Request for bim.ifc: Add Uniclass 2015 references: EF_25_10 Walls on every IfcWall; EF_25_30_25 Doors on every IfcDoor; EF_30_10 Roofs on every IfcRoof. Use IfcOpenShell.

First a look at what the model holds.

```python
import ifcopenshell

model = ifcopenshell.open("bim.ifc")
print(model.schema)
print("classifications:", [c.Name for c in model.by_type("IfcClassification")])
for ifc_class in ("IfcDoor", "IfcRoof", "IfcStair", "IfcWall", "IfcWindow"):
    print(ifc_class, len(model.by_type(ifc_class)))
```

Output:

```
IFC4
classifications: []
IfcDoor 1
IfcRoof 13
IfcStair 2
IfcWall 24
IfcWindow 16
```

```python
import ifcopenshell
import ifcopenshell.api.classification

model = ifcopenshell.open("bim.ifc")

system = ifcopenshell.api.classification.add_classification(model, classification="Uniclass 2015")

codes = {
    "IfcWall": ("EF_25_10", "Walls"),
    "IfcDoor": ("EF_25_30_25", "Doors"),
    "IfcRoof": ("EF_30_10", "Roofs"),
}
for ifc_class, (code, name) in codes.items():
    products = model.by_type(ifc_class)
    ifcopenshell.api.classification.add_reference(
        model, products=products, classification=system, identification=code, name=name
    )
    print(code, len(products))

model.write("bim_v2.ifc")
```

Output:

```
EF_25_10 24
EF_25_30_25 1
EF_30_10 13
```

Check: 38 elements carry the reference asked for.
